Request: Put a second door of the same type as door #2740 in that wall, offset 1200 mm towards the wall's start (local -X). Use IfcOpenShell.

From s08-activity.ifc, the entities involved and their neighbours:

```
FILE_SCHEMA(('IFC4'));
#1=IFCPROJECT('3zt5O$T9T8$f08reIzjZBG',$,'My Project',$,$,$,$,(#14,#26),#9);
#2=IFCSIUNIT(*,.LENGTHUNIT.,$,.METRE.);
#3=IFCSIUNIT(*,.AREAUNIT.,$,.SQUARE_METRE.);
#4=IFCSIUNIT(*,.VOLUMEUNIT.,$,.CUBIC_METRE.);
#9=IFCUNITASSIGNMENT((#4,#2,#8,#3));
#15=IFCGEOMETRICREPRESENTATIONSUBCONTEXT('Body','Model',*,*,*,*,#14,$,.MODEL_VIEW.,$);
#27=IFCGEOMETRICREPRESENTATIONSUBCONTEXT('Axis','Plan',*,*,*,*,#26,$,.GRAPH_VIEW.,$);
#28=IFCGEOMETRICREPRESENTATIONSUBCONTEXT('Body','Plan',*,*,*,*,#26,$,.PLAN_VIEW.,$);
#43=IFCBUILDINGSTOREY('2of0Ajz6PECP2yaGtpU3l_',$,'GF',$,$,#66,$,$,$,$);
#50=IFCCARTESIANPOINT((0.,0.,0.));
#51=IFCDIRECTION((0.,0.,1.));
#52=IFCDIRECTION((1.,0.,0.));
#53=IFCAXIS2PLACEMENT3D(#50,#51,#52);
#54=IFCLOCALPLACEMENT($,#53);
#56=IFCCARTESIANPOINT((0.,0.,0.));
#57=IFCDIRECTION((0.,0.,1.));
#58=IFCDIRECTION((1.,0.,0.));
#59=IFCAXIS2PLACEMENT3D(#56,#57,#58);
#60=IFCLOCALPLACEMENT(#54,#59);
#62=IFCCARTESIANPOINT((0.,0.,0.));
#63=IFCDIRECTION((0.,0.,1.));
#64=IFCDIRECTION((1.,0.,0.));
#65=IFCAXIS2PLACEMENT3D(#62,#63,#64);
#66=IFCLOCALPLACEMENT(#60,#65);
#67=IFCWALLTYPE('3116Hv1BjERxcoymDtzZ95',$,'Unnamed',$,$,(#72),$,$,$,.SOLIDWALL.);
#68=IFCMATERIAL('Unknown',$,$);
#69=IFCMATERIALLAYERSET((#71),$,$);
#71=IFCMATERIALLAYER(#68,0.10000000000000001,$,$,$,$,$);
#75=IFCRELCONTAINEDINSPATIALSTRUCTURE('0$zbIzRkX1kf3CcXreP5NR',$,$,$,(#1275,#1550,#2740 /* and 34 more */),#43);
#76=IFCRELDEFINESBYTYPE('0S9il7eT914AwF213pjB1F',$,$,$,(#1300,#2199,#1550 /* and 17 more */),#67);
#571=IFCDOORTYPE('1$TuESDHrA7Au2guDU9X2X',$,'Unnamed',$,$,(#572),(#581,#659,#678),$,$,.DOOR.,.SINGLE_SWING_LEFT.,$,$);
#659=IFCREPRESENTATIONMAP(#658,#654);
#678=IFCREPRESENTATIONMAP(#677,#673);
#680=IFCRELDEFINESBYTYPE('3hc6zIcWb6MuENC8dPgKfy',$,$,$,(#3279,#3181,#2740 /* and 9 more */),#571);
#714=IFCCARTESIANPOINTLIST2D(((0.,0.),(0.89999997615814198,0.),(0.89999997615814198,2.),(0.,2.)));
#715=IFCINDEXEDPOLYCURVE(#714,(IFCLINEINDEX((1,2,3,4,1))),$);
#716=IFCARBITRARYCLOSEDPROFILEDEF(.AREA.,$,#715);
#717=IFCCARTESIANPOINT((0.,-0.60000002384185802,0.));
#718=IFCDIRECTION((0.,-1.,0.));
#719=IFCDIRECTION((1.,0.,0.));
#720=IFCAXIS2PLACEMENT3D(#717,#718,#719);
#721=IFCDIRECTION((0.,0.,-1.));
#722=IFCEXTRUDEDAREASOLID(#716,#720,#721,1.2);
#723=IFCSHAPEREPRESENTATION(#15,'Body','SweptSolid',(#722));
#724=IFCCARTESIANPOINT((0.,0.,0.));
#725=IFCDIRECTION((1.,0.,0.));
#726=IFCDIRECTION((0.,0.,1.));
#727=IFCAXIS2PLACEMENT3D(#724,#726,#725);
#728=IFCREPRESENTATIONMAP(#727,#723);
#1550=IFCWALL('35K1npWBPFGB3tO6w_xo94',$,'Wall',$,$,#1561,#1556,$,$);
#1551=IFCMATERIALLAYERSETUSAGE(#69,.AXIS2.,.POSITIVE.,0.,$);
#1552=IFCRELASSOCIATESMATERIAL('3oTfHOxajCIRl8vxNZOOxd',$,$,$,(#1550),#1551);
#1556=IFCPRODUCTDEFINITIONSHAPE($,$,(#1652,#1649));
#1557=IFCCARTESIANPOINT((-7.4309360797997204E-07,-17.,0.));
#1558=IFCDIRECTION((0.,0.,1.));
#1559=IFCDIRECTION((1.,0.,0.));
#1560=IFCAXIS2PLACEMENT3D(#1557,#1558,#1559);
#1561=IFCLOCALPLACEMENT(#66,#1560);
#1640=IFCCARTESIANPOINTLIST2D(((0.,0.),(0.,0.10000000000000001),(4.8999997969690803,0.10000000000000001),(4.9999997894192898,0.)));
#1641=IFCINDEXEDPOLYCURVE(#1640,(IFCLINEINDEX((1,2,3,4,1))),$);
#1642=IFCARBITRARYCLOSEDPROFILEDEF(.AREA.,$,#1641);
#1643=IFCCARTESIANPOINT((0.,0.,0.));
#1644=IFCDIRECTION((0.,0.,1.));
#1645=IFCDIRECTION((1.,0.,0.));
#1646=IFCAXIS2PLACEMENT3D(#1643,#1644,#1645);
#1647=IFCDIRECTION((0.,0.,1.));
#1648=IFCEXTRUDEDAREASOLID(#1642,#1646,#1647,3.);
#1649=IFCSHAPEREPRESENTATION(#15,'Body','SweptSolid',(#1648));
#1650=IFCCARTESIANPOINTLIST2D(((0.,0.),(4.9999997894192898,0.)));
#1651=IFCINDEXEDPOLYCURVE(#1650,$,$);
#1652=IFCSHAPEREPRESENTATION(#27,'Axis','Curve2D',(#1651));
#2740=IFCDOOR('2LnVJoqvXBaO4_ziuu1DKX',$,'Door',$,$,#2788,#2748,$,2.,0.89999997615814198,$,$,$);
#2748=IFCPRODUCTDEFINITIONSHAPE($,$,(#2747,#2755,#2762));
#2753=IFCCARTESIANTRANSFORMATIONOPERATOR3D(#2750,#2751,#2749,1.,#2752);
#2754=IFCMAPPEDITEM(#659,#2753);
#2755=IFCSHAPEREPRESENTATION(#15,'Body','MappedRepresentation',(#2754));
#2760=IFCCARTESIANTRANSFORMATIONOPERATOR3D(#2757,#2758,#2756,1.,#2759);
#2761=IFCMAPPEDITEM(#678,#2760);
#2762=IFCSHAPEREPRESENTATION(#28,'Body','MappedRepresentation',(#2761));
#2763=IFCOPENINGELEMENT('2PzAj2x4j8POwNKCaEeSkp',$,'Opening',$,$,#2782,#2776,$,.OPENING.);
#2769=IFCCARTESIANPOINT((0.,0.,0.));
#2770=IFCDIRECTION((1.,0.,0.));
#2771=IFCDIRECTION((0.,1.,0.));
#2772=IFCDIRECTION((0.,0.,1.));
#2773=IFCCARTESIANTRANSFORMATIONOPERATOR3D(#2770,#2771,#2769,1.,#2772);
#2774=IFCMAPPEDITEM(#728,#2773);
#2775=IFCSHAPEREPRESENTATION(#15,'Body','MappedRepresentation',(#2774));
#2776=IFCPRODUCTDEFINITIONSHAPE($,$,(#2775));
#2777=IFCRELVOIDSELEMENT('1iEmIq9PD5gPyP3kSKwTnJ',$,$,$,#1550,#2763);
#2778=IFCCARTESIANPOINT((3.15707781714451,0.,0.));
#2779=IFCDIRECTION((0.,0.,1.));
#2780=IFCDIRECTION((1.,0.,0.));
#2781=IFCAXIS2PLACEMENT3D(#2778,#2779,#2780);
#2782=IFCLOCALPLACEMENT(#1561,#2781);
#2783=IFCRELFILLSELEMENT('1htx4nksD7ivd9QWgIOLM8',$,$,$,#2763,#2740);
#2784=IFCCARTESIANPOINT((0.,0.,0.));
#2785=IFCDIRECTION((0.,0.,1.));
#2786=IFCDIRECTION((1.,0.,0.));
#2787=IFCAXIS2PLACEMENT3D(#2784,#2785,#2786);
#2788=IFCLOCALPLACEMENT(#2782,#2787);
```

```python
import ifcopenshell
import ifcopenshell.api.feature
import ifcopenshell.api.geometry
import ifcopenshell.api.root
import ifcopenshell.geom
import ifcopenshell.util.element
import ifcopenshell.util.placement
import ifcopenshell.util.shape
import ifcopenshell.util.unit

model = ifcopenshell.open("s08-activity.ifc")
unit_scale = ifcopenshell.util.unit.calculate_unit_scale(model)
settings = ifcopenshell.geom.settings()


def volume(element):
    """Net volume in cubic metres, openings subtracted."""
    shape = ifcopenshell.geom.create_shape(settings, element)
    return ifcopenshell.util.shape.get_volume(shape.geometry)


door = model.by_guid("2LnVJoqvXBaO4_ziuu1DKX")
opening = door.FillsVoids[0].RelatingOpeningElement
wall = opening.VoidsElements[0].RelatingBuildingElement
before = volume(wall)
shift = ifcopenshell.util.placement.get_local_placement(wall.ObjectPlacement)[:3, 0] * -1.2 / unit_scale

# copy_class copies the void relationship, type, container and properties, but no geometry.
new_opening = ifcopenshell.api.root.copy_class(model, product=opening)
new_opening.Representation = ifcopenshell.util.element.copy_deep(
    model, opening.Representation, exclude=["IfcGeometricRepresentationContext", "IfcRepresentationMap"]
)
new_door = ifcopenshell.api.root.copy_class(model, product=door)
new_door.Representation = ifcopenshell.util.element.copy_deep(
    model, door.Representation, exclude=["IfcGeometricRepresentationContext", "IfcRepresentationMap"]
)
ifcopenshell.api.feature.add_filling(model, opening=new_opening, element=new_door)

for old, new in ((opening, new_opening), (door, new_door)):
    matrix = ifcopenshell.util.placement.get_local_placement(old.ObjectPlacement)
    matrix[:3, 3] += shift
    ifcopenshell.api.geometry.edit_object_placement(model, product=new, matrix=matrix, is_si=False)

after = volume(wall)

print(f"wall volume {before:.3f} -> {after:.3f} m3")

model.write("s08-activity_edited.ifc")
```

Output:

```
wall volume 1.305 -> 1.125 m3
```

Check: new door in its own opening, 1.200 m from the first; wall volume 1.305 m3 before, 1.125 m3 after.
